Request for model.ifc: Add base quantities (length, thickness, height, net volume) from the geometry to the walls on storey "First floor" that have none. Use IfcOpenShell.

First a look at what the model holds.

```python
import ifcopenshell
import ifcopenshell.util.element
import ifcopenshell.util.unit

model = ifcopenshell.open("model.ifc")
print(model.schema)
for unit_type in ("LENGTHUNIT", "AREAUNIT", "VOLUMEUNIT"):
    print(unit_type, ifcopenshell.util.unit.calculate_unit_scale(model, unit_type))
storey = next(s for s in model.by_type("IfcBuildingStorey") if s.Name == "First floor")
walls = [e for e in ifcopenshell.util.element.get_decomposition(storey) if e.is_a("IfcWall")]
for e in sorted(walls, key=lambda e: e.id()):
    print(e.id(), e.is_a(), e.Name, list(ifcopenshell.util.element.get_psets(e, qtos_only=True)), sep=" | ")
```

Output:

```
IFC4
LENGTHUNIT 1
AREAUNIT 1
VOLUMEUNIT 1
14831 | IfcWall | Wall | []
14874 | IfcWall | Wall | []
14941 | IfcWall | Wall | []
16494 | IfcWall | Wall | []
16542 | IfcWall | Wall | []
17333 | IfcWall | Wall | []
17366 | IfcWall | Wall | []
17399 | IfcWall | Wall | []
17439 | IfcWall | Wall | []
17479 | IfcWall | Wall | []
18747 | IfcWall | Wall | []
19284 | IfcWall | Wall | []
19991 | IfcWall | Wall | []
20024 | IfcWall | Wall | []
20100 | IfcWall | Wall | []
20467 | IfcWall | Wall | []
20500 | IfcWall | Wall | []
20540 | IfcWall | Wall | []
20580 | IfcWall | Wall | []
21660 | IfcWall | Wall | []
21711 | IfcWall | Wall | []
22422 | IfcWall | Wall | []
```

```python
import ifcopenshell
import ifcopenshell.api.pset
import ifcopenshell.geom
import ifcopenshell.util.element
import ifcopenshell.util.shape
import ifcopenshell.util.unit

model = ifcopenshell.open("model.ifc")
unit_scale = ifcopenshell.util.unit.calculate_unit_scale(model)
volume_scale = ifcopenshell.util.unit.calculate_unit_scale(model, "VOLUMEUNIT")
settings = ifcopenshell.geom.settings()

storey = next(s for s in model.by_type("IfcBuildingStorey") if s.Name == "First floor")
walls = [e for e in ifcopenshell.util.element.get_decomposition(storey) if e.is_a("IfcWall")]

for e in sorted(walls, key=lambda e: e.id()):
    if ifcopenshell.util.element.get_psets(e, qtos_only=True, should_inherit=False):
        continue
    # Geometry comes back in metres, in the element's own axes.
    shape = ifcopenshell.geom.create_shape(settings, e)
    values = {
        "Length": ifcopenshell.util.shape.get_x(shape.geometry) / unit_scale,
        "Width": ifcopenshell.util.shape.get_y(shape.geometry) / unit_scale,
        "Height": ifcopenshell.util.shape.get_z(shape.geometry) / unit_scale,
        "NetVolume": ifcopenshell.util.shape.get_volume(shape.geometry) / volume_scale,
    }
    qto = ifcopenshell.api.pset.add_qto(model, product=e, name="Qto_WallBaseQuantities")
    ifcopenshell.api.pset.edit_qto(model, qto=qto, properties=values)
    print(e.id(), {k: round(v, 3) for k, v in values.items()})

model.write("model_v2.ifc")
```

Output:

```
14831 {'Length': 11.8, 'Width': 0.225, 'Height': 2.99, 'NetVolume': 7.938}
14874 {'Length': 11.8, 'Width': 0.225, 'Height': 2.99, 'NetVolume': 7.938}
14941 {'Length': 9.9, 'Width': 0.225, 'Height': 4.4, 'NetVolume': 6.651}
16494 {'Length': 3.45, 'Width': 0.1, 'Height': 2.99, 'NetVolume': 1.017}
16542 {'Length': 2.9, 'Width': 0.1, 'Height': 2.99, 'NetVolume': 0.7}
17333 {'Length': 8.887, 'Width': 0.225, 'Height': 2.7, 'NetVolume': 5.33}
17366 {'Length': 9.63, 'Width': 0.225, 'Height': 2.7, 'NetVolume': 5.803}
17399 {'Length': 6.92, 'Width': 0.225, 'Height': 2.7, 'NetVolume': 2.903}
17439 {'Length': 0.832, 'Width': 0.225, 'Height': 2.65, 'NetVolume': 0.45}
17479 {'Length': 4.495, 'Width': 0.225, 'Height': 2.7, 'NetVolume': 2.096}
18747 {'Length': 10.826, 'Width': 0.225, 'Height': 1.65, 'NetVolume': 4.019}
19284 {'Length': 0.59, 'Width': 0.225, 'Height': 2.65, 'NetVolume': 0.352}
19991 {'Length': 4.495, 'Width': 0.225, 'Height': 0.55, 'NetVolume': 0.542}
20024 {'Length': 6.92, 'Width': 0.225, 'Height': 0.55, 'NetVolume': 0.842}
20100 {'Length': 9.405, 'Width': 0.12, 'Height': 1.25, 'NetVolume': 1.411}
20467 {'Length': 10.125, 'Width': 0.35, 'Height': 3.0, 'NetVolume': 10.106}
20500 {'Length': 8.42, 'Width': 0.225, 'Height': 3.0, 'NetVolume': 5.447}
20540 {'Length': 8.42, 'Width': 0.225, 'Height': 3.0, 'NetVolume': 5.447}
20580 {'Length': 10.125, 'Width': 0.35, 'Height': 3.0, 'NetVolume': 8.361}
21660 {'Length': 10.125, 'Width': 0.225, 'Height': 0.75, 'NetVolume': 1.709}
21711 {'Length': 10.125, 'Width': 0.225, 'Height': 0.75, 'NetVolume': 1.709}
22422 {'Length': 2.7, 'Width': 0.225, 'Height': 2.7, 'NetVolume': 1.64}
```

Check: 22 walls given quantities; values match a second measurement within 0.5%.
